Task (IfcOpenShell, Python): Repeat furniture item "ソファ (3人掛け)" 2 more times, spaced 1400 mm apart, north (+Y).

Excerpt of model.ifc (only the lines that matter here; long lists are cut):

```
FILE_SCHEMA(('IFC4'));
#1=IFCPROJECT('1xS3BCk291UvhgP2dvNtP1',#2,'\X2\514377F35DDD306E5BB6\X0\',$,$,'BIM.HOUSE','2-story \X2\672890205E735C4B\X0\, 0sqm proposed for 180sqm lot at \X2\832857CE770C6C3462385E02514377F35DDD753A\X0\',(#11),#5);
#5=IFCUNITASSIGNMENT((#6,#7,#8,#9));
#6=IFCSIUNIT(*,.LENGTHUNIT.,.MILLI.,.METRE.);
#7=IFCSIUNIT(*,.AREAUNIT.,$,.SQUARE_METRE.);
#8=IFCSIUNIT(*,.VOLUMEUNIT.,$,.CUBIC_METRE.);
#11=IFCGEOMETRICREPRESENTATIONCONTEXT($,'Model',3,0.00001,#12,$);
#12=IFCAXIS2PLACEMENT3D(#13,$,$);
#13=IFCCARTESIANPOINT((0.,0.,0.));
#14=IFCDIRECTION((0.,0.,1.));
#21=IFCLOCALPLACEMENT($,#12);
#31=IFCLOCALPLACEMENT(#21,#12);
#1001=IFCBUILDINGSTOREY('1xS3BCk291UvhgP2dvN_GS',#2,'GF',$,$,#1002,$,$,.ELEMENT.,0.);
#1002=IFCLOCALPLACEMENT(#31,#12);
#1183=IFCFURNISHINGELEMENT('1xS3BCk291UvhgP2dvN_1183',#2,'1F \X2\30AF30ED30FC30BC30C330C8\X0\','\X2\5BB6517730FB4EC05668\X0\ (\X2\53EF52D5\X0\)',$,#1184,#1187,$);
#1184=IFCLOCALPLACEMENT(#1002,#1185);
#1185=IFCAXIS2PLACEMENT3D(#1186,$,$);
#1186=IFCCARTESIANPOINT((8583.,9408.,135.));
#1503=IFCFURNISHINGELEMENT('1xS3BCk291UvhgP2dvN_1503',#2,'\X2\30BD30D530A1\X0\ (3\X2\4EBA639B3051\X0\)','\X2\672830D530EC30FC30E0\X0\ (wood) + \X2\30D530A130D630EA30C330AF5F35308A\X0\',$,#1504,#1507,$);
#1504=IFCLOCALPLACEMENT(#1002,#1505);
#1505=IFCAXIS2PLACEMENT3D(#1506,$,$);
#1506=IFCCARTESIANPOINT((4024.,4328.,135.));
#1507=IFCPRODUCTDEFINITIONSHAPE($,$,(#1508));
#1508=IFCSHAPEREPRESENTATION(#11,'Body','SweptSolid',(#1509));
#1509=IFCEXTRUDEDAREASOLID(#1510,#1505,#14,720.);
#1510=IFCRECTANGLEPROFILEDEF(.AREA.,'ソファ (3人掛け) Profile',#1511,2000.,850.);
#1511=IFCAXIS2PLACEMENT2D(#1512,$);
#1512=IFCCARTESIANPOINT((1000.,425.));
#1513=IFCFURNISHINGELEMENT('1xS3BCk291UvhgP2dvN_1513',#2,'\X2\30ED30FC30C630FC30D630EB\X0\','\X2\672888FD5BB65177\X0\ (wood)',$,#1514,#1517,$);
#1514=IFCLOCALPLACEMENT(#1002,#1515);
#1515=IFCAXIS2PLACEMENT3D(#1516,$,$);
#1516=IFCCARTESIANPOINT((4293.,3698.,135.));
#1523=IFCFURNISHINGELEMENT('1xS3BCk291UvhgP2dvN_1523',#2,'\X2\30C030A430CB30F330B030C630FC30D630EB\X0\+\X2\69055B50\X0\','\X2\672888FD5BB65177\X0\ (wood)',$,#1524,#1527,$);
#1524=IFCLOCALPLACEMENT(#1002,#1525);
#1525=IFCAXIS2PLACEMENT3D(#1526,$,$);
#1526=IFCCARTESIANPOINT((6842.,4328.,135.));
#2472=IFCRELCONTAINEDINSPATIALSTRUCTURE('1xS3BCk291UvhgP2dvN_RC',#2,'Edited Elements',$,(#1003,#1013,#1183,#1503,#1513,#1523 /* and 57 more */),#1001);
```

```python
import numpy as np
import ifcopenshell
import ifcopenshell.api.geometry
import ifcopenshell.api.root
import ifcopenshell.util.element
import ifcopenshell.util.placement
import ifcopenshell.util.unit

model = ifcopenshell.open("model.ifc")
unit_scale = ifcopenshell.util.unit.calculate_unit_scale(model)


def reuse_history(source, copy):
    """copy_class also copies each property set's owner history, people and application; keep the originals."""
    for rel in copy.IsDefinedBy:
        if rel.is_a("IfcRelDefinesByProperties") and (history := rel.RelatingPropertyDefinition.OwnerHistory):
            rel.RelatingPropertyDefinition.OwnerHistory = source.OwnerHistory
            ifcopenshell.util.element.remove_deep2(model, history)


source = model.by_guid("1xS3BCk291UvhgP2dvN_1503")
base = ifcopenshell.util.placement.get_local_placement(source.ObjectPlacement)
step = np.array([0.0, 1.0, 0.0]) * 1.4 / unit_scale

for i in range(1, 3):
    copy = ifcopenshell.api.root.copy_class(model, product=source)
    copy.Representation = ifcopenshell.util.element.copy_deep(
        model, source.Representation, exclude=["IfcGeometricRepresentationContext", "IfcRepresentationMap"]
    )
    reuse_history(source, copy)
    matrix = base.copy()
    matrix[:3, 3] += i * step
    print("added at", matrix[:3, 3].round(3) + 0.0)
    ifcopenshell.api.geometry.edit_object_placement(model, product=copy, matrix=matrix, is_si=False)

model.write("model_rev.ifc")
```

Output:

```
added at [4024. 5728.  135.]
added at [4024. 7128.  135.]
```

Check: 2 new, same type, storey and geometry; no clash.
